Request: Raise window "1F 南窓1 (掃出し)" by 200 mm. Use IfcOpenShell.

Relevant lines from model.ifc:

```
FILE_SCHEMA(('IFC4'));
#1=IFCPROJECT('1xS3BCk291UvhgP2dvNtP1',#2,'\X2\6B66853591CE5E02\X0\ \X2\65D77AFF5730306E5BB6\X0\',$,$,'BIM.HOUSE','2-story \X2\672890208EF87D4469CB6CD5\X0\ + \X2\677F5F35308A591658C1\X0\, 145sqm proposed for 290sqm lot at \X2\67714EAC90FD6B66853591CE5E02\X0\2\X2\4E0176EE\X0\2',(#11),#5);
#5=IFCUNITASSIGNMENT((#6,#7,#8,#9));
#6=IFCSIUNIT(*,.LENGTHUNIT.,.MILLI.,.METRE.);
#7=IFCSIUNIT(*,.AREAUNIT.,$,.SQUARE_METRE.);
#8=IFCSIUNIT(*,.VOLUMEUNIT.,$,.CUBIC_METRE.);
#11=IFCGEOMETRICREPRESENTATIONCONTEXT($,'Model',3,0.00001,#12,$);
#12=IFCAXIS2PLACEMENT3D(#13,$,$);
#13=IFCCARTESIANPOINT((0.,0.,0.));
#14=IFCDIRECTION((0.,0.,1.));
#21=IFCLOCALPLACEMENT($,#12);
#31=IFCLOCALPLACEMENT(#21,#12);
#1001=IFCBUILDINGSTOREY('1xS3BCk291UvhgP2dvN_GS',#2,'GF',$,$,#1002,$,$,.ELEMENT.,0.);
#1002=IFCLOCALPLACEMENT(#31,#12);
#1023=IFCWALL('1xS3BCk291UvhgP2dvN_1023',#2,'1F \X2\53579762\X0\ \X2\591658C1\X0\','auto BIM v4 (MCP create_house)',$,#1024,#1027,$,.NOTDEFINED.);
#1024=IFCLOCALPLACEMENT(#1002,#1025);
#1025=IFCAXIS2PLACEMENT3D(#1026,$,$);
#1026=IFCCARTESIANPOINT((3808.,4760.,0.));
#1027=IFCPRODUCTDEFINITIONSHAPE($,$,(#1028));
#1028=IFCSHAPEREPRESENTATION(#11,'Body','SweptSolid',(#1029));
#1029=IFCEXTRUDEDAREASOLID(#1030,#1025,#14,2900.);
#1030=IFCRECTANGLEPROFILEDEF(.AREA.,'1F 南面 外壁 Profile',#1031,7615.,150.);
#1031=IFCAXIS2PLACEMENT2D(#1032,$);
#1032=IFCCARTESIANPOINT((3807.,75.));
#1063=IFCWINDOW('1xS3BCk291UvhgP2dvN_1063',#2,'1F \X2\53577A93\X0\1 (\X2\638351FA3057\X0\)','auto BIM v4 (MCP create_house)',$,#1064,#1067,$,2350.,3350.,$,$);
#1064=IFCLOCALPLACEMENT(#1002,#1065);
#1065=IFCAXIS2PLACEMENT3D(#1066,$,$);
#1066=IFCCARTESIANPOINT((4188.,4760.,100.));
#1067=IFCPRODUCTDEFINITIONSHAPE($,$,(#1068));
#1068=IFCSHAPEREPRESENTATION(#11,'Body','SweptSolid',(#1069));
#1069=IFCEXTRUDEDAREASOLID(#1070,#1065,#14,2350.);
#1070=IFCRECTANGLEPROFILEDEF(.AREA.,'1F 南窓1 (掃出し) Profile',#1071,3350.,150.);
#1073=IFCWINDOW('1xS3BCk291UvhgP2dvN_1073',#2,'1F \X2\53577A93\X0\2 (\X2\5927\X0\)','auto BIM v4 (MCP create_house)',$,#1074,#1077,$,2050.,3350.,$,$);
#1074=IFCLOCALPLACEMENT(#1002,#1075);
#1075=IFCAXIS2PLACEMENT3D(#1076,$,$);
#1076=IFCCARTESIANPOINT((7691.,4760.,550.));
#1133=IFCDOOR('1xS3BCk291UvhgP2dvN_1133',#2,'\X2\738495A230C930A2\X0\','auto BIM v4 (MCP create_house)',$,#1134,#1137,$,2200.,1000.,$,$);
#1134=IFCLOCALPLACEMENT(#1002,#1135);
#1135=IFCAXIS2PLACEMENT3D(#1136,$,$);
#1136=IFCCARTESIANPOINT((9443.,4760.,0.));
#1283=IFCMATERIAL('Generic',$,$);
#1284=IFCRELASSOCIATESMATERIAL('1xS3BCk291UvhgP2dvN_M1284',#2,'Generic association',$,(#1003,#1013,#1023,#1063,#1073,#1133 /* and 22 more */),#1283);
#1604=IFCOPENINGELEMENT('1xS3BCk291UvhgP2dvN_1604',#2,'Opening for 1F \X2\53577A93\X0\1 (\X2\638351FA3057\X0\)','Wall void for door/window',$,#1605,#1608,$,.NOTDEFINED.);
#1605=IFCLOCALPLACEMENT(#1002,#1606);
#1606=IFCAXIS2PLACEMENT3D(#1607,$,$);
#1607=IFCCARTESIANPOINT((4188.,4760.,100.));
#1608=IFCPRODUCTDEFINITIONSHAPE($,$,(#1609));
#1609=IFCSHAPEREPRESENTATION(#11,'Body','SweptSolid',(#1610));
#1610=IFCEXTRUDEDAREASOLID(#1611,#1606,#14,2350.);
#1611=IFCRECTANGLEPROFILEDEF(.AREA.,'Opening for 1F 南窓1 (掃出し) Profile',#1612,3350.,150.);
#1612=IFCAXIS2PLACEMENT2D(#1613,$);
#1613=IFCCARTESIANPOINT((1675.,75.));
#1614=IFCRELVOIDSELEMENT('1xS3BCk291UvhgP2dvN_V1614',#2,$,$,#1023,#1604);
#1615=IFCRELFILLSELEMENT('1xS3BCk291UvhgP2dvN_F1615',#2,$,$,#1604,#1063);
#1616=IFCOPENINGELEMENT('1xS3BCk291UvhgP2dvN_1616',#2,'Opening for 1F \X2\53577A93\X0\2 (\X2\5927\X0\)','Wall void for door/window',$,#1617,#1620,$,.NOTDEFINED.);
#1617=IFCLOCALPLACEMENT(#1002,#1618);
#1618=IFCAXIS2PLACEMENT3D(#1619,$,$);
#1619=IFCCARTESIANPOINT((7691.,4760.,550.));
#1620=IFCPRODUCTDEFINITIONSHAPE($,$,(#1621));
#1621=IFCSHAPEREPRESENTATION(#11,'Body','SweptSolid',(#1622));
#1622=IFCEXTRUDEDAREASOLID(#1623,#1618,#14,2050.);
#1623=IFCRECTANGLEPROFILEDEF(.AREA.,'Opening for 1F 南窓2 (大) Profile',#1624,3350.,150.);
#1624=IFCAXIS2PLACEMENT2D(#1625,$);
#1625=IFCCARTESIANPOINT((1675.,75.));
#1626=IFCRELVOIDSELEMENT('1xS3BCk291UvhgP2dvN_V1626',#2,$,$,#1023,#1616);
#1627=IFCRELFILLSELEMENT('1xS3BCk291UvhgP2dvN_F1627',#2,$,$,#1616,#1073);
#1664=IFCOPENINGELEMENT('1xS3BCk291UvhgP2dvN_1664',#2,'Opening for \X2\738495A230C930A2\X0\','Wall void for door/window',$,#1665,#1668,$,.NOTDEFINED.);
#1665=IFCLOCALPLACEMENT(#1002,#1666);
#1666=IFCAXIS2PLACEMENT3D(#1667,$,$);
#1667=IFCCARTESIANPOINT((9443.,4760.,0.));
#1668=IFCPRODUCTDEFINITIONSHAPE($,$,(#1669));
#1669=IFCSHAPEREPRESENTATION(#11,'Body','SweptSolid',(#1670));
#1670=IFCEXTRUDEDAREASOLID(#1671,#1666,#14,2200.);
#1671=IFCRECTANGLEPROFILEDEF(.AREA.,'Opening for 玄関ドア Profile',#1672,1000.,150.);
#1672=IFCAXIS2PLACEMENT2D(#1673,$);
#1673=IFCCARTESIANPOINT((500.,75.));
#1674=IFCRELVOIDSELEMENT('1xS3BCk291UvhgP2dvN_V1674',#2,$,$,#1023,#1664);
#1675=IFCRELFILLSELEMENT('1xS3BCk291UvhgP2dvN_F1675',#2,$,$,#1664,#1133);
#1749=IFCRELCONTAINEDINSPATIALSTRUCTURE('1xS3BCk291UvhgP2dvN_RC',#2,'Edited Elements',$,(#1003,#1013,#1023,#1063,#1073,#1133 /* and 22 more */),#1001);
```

```python
import numpy as np
import ifcopenshell
import ifcopenshell.api.geometry
import ifcopenshell.util.placement
import ifcopenshell.util.unit

model = ifcopenshell.open("model.ifc")
unit_scale = ifcopenshell.util.unit.calculate_unit_scale(model)

window = model.by_guid("1xS3BCk291UvhgP2dvN_1063")
opening = window.FillsVoids[0].RelatingOpeningElement
dz = 0.2 / unit_scale

shift = np.array([0.0, 0.0, dz])
# The window is not placed relative to its opening, so move both.
for product in (opening, window):
    matrix = ifcopenshell.util.placement.get_local_placement(product.ObjectPlacement)
    matrix[:3, 3] += shift
    ifcopenshell.api.geometry.edit_object_placement(model, product=product, matrix=matrix, is_si=False)

print(f"moved by {dz * unit_scale:+.3f} m")

model.write("model-out.ifc")
```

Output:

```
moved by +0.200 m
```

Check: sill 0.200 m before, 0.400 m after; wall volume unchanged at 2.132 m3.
